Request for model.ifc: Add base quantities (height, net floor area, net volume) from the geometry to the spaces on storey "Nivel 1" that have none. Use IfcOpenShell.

First a look at what the model holds.

```python
import ifcopenshell
import ifcopenshell.util.element
import ifcopenshell.util.unit

model = ifcopenshell.open("model.ifc")
print(model.schema)
for unit_type in ("LENGTHUNIT", "AREAUNIT", "VOLUMEUNIT"):
    print(unit_type, ifcopenshell.util.unit.calculate_unit_scale(model, unit_type))
storey = next(s for s in model.by_type("IfcBuildingStorey") if s.Name == "Nivel 1")
spaces = [e for e in ifcopenshell.util.element.get_decomposition(storey) if e.is_a("IfcSpace")]
for e in sorted(spaces, key=lambda e: e.id()):
    print(e.id(), e.is_a(), e.Name, list(ifcopenshell.util.element.get_psets(e, qtos_only=True)), sep=" | ")
```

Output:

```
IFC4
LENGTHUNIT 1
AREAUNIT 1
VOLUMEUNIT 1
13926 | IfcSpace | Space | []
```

```python
import ifcopenshell
import ifcopenshell.api.pset
import ifcopenshell.geom
import ifcopenshell.util.element
import ifcopenshell.util.shape
import ifcopenshell.util.unit

model = ifcopenshell.open("model.ifc")
unit_scale = ifcopenshell.util.unit.calculate_unit_scale(model)
area_scale = ifcopenshell.util.unit.calculate_unit_scale(model, "AREAUNIT")
volume_scale = ifcopenshell.util.unit.calculate_unit_scale(model, "VOLUMEUNIT")
settings = ifcopenshell.geom.settings()

storey = next(s for s in model.by_type("IfcBuildingStorey") if s.Name == "Nivel 1")
spaces = [e for e in ifcopenshell.util.element.get_decomposition(storey) if e.is_a("IfcSpace")]

for e in sorted(spaces, key=lambda e: e.id()):
    if ifcopenshell.util.element.get_psets(e, qtos_only=True, should_inherit=False):
        continue
    # Geometry comes back in metres, in the element's own axes.
    shape = ifcopenshell.geom.create_shape(settings, e)
    values = {
        "Height": ifcopenshell.util.shape.get_z(shape.geometry) / unit_scale,
        "NetFloorArea": ifcopenshell.util.shape.get_footprint_area(shape.geometry) / area_scale,
        "NetVolume": ifcopenshell.util.shape.get_volume(shape.geometry) / volume_scale,
    }
    qto = ifcopenshell.api.pset.add_qto(model, product=e, name="Qto_SpaceBaseQuantities")
    ifcopenshell.api.pset.edit_qto(model, qto=qto, properties=values)
    print(e.id(), {k: round(v, 3) for k, v in values.items()})

model.write("model_v2.ifc")
```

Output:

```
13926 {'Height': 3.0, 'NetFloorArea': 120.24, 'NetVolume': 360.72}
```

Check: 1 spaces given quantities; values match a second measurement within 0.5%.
